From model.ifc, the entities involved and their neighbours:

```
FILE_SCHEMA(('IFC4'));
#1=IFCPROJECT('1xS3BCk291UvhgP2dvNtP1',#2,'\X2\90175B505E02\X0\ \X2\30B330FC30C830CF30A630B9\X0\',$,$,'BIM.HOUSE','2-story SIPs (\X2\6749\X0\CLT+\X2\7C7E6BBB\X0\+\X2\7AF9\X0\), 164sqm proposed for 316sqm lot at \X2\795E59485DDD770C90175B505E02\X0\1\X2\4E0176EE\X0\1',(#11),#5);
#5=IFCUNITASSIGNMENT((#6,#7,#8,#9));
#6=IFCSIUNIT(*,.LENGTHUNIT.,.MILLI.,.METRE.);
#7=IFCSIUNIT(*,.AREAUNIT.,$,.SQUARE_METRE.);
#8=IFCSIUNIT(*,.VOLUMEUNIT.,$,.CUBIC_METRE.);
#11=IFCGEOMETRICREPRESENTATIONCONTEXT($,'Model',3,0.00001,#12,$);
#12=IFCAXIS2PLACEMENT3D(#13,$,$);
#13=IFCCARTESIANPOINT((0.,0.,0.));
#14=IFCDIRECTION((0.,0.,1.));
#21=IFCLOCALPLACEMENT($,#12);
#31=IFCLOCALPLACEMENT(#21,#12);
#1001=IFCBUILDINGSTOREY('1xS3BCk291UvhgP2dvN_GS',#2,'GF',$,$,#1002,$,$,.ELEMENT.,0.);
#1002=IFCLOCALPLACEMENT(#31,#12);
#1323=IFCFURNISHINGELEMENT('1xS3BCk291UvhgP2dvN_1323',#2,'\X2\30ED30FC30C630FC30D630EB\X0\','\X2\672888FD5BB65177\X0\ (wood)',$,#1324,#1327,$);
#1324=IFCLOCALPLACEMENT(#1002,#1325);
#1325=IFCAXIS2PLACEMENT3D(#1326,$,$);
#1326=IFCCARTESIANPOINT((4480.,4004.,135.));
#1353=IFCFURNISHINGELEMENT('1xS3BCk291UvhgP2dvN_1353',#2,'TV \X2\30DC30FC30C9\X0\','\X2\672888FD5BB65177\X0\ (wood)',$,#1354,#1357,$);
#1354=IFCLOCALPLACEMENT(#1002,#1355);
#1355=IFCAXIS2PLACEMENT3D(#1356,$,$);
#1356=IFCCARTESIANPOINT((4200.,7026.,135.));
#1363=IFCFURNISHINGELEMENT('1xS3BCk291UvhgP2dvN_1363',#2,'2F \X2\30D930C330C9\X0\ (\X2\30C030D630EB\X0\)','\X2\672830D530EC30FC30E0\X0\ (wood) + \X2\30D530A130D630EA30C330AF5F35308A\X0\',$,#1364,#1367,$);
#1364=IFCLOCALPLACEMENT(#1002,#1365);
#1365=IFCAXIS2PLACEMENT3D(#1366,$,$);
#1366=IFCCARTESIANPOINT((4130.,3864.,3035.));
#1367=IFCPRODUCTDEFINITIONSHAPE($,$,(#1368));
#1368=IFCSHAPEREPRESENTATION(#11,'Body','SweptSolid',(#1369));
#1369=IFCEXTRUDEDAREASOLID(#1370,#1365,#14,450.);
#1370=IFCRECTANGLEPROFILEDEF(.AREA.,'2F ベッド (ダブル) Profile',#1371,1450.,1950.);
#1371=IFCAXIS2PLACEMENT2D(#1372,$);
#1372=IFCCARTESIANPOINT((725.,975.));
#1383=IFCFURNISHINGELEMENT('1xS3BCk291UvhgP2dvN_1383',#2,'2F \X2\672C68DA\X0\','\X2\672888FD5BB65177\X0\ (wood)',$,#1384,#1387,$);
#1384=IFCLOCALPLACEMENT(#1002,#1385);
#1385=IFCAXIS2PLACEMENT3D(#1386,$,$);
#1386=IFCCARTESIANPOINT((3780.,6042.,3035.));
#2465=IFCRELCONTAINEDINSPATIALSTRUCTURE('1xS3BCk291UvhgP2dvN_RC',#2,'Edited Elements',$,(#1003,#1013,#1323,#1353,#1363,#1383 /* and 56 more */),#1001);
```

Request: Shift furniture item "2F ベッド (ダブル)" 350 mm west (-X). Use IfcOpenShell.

```python
import ifcopenshell
import ifcopenshell.api.geometry
import ifcopenshell.util.placement
import ifcopenshell.util.unit

model = ifcopenshell.open("model.ifc")
unit_scale = ifcopenshell.util.unit.calculate_unit_scale(model)

item = model.by_id(1363)
matrix = ifcopenshell.util.placement.get_local_placement(item.ObjectPlacement)
matrix[0, 3] -= 0.35 / unit_scale
ifcopenshell.api.geometry.edit_object_placement(model, product=item, matrix=matrix, is_si=False)

print(ifcopenshell.util.placement.get_local_placement(item.ObjectPlacement).round(3) + 0.0)

model.write("model_updated.ifc")
```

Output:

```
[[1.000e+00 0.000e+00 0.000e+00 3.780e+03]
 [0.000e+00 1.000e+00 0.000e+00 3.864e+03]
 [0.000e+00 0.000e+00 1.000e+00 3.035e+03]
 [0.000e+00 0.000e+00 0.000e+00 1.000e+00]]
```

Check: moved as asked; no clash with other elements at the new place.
